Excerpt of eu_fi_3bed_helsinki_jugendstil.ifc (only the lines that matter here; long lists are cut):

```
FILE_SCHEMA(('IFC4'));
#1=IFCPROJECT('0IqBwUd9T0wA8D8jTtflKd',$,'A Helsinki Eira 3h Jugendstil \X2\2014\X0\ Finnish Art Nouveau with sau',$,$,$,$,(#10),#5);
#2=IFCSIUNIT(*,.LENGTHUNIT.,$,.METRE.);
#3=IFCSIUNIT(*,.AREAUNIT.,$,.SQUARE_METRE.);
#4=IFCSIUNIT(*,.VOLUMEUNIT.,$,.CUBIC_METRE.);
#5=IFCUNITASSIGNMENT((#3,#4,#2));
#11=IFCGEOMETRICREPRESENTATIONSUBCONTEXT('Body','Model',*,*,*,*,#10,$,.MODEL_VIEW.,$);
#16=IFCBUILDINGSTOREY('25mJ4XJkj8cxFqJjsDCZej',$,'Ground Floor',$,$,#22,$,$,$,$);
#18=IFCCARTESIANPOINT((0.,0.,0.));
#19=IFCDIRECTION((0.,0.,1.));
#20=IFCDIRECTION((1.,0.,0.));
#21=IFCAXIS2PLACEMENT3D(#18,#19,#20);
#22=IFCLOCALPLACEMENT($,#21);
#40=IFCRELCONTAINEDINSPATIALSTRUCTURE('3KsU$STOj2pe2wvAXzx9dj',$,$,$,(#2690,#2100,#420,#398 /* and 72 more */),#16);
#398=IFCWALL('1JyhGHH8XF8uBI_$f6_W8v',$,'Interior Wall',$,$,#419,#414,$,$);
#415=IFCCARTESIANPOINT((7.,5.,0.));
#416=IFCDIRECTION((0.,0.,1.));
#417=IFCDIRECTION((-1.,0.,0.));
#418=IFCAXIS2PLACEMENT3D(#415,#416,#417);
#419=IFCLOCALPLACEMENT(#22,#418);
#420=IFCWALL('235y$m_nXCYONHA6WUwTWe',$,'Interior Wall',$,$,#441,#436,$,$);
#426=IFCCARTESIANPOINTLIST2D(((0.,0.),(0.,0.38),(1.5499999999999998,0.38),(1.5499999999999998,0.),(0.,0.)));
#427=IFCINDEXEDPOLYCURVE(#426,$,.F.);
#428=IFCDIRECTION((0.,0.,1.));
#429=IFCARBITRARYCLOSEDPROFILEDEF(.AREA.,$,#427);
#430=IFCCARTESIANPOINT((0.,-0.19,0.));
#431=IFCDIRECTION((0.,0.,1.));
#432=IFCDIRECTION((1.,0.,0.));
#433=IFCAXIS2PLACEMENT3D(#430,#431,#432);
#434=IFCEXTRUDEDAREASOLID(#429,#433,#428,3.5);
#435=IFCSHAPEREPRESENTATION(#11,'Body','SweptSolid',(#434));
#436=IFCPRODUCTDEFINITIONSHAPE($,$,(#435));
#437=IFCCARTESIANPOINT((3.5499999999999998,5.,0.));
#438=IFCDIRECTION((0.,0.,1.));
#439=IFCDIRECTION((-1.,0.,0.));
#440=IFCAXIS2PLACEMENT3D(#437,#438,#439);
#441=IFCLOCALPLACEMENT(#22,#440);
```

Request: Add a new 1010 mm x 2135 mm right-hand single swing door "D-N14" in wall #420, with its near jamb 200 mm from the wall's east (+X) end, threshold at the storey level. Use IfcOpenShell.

```python
import numpy as np
import ifcopenshell
import ifcopenshell.api.feature
import ifcopenshell.api.geometry
import ifcopenshell.api.root
import ifcopenshell.api.spatial
import ifcopenshell.geom
import ifcopenshell.util.element
import ifcopenshell.util.placement
import ifcopenshell.util.representation
import ifcopenshell.util.shape
import ifcopenshell.util.unit

model = ifcopenshell.open("eu_fi_3bed_helsinki_jugendstil.ifc")
unit_scale = ifcopenshell.util.unit.calculate_unit_scale(model)
settings = ifcopenshell.geom.settings()


def volume(element):
    """Net volume in cubic metres, openings subtracted."""
    shape = ifcopenshell.geom.create_shape(settings, element)
    return ifcopenshell.util.shape.get_volume(shape.geometry)


wall = model.by_id(420)
storey = ifcopenshell.util.element.get_container(wall, ifc_class="IfcBuildingStorey")
context = ifcopenshell.util.representation.get_context(model, "Model", "Body", "MODEL_VIEW")
before = volume(wall)

width, height, from_end, sill = 1.01, 2.135, 0.2, 0.0  # metres

# The wall runs along its own X axis, and the end named is its -X end.
wall_shape = ifcopenshell.geom.create_shape(settings, wall)
x, y, z = ifcopenshell.util.shape.get_vertices(wall_shape.geometry).T
start = x.min() + from_end
face, thickness = float(y.min()), float(y.max() - y.min())
wall_matrix = ifcopenshell.util.placement.get_local_placement(wall.ObjectPlacement)
level = ifcopenshell.util.placement.get_local_placement(storey.ObjectPlacement)[2, 3]


def in_wall(x, y):
    """Placement at x, y metres in the wall's axes, at sill height."""
    matrix = wall_matrix.copy()
    matrix[:, 3] = wall_matrix @ np.array([x / unit_scale, y / unit_scale, 0.0, 1.0])
    matrix[2, 3] = level + sill / unit_scale
    return matrix


# Opening: a box that overshoots both wall faces by 50 mm.
opening = ifcopenshell.api.root.create_entity(model, ifc_class="IfcOpeningElement", predefined_type="OPENING")
box = ifcopenshell.api.geometry.add_wall_representation(
    model, context=context, length=width, height=height, thickness=thickness + 0.1
)
ifcopenshell.api.geometry.assign_representation(model, product=opening, representation=box)
ifcopenshell.api.geometry.edit_object_placement(model, product=opening, matrix=in_wall(start, face - 0.05), is_si=False)
ifcopenshell.api.feature.add_feature(model, feature=opening, element=wall)

door = ifcopenshell.api.root.create_entity(model, ifc_class="IfcDoor", name="D-N14", predefined_type="DOOR")
door.OverallWidth, door.OverallHeight = width / unit_scale, height / unit_scale
door.OperationType = "SINGLE_SWING_RIGHT"
body = ifcopenshell.api.geometry.add_door_representation(
    model,
    context=context,
    overall_width=door.OverallWidth,
    overall_height=door.OverallHeight,
    operation_type="SINGLE_SWING_RIGHT",
    lining_properties={"LiningDepth": thickness / unit_scale, "ThresholdDepth": thickness / unit_scale},
)
ifcopenshell.api.geometry.assign_representation(model, product=door, representation=body)
ifcopenshell.api.spatial.assign_container(model, products=[door], relating_structure=storey)
ifcopenshell.api.feature.add_filling(model, opening=opening, element=door)

# The lining spans the wall, so the door starts at the wall face.
ifcopenshell.api.geometry.edit_object_placement(model, product=door, matrix=in_wall(start, face), is_si=False)

after = volume(wall)

print(f"wall volume {before:.3f} -> {after:.3f} m3")

model.write("eu_fi_3bed_helsinki_jugendstil_v2.ifc")
```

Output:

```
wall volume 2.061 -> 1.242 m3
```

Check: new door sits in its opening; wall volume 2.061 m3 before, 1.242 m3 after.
